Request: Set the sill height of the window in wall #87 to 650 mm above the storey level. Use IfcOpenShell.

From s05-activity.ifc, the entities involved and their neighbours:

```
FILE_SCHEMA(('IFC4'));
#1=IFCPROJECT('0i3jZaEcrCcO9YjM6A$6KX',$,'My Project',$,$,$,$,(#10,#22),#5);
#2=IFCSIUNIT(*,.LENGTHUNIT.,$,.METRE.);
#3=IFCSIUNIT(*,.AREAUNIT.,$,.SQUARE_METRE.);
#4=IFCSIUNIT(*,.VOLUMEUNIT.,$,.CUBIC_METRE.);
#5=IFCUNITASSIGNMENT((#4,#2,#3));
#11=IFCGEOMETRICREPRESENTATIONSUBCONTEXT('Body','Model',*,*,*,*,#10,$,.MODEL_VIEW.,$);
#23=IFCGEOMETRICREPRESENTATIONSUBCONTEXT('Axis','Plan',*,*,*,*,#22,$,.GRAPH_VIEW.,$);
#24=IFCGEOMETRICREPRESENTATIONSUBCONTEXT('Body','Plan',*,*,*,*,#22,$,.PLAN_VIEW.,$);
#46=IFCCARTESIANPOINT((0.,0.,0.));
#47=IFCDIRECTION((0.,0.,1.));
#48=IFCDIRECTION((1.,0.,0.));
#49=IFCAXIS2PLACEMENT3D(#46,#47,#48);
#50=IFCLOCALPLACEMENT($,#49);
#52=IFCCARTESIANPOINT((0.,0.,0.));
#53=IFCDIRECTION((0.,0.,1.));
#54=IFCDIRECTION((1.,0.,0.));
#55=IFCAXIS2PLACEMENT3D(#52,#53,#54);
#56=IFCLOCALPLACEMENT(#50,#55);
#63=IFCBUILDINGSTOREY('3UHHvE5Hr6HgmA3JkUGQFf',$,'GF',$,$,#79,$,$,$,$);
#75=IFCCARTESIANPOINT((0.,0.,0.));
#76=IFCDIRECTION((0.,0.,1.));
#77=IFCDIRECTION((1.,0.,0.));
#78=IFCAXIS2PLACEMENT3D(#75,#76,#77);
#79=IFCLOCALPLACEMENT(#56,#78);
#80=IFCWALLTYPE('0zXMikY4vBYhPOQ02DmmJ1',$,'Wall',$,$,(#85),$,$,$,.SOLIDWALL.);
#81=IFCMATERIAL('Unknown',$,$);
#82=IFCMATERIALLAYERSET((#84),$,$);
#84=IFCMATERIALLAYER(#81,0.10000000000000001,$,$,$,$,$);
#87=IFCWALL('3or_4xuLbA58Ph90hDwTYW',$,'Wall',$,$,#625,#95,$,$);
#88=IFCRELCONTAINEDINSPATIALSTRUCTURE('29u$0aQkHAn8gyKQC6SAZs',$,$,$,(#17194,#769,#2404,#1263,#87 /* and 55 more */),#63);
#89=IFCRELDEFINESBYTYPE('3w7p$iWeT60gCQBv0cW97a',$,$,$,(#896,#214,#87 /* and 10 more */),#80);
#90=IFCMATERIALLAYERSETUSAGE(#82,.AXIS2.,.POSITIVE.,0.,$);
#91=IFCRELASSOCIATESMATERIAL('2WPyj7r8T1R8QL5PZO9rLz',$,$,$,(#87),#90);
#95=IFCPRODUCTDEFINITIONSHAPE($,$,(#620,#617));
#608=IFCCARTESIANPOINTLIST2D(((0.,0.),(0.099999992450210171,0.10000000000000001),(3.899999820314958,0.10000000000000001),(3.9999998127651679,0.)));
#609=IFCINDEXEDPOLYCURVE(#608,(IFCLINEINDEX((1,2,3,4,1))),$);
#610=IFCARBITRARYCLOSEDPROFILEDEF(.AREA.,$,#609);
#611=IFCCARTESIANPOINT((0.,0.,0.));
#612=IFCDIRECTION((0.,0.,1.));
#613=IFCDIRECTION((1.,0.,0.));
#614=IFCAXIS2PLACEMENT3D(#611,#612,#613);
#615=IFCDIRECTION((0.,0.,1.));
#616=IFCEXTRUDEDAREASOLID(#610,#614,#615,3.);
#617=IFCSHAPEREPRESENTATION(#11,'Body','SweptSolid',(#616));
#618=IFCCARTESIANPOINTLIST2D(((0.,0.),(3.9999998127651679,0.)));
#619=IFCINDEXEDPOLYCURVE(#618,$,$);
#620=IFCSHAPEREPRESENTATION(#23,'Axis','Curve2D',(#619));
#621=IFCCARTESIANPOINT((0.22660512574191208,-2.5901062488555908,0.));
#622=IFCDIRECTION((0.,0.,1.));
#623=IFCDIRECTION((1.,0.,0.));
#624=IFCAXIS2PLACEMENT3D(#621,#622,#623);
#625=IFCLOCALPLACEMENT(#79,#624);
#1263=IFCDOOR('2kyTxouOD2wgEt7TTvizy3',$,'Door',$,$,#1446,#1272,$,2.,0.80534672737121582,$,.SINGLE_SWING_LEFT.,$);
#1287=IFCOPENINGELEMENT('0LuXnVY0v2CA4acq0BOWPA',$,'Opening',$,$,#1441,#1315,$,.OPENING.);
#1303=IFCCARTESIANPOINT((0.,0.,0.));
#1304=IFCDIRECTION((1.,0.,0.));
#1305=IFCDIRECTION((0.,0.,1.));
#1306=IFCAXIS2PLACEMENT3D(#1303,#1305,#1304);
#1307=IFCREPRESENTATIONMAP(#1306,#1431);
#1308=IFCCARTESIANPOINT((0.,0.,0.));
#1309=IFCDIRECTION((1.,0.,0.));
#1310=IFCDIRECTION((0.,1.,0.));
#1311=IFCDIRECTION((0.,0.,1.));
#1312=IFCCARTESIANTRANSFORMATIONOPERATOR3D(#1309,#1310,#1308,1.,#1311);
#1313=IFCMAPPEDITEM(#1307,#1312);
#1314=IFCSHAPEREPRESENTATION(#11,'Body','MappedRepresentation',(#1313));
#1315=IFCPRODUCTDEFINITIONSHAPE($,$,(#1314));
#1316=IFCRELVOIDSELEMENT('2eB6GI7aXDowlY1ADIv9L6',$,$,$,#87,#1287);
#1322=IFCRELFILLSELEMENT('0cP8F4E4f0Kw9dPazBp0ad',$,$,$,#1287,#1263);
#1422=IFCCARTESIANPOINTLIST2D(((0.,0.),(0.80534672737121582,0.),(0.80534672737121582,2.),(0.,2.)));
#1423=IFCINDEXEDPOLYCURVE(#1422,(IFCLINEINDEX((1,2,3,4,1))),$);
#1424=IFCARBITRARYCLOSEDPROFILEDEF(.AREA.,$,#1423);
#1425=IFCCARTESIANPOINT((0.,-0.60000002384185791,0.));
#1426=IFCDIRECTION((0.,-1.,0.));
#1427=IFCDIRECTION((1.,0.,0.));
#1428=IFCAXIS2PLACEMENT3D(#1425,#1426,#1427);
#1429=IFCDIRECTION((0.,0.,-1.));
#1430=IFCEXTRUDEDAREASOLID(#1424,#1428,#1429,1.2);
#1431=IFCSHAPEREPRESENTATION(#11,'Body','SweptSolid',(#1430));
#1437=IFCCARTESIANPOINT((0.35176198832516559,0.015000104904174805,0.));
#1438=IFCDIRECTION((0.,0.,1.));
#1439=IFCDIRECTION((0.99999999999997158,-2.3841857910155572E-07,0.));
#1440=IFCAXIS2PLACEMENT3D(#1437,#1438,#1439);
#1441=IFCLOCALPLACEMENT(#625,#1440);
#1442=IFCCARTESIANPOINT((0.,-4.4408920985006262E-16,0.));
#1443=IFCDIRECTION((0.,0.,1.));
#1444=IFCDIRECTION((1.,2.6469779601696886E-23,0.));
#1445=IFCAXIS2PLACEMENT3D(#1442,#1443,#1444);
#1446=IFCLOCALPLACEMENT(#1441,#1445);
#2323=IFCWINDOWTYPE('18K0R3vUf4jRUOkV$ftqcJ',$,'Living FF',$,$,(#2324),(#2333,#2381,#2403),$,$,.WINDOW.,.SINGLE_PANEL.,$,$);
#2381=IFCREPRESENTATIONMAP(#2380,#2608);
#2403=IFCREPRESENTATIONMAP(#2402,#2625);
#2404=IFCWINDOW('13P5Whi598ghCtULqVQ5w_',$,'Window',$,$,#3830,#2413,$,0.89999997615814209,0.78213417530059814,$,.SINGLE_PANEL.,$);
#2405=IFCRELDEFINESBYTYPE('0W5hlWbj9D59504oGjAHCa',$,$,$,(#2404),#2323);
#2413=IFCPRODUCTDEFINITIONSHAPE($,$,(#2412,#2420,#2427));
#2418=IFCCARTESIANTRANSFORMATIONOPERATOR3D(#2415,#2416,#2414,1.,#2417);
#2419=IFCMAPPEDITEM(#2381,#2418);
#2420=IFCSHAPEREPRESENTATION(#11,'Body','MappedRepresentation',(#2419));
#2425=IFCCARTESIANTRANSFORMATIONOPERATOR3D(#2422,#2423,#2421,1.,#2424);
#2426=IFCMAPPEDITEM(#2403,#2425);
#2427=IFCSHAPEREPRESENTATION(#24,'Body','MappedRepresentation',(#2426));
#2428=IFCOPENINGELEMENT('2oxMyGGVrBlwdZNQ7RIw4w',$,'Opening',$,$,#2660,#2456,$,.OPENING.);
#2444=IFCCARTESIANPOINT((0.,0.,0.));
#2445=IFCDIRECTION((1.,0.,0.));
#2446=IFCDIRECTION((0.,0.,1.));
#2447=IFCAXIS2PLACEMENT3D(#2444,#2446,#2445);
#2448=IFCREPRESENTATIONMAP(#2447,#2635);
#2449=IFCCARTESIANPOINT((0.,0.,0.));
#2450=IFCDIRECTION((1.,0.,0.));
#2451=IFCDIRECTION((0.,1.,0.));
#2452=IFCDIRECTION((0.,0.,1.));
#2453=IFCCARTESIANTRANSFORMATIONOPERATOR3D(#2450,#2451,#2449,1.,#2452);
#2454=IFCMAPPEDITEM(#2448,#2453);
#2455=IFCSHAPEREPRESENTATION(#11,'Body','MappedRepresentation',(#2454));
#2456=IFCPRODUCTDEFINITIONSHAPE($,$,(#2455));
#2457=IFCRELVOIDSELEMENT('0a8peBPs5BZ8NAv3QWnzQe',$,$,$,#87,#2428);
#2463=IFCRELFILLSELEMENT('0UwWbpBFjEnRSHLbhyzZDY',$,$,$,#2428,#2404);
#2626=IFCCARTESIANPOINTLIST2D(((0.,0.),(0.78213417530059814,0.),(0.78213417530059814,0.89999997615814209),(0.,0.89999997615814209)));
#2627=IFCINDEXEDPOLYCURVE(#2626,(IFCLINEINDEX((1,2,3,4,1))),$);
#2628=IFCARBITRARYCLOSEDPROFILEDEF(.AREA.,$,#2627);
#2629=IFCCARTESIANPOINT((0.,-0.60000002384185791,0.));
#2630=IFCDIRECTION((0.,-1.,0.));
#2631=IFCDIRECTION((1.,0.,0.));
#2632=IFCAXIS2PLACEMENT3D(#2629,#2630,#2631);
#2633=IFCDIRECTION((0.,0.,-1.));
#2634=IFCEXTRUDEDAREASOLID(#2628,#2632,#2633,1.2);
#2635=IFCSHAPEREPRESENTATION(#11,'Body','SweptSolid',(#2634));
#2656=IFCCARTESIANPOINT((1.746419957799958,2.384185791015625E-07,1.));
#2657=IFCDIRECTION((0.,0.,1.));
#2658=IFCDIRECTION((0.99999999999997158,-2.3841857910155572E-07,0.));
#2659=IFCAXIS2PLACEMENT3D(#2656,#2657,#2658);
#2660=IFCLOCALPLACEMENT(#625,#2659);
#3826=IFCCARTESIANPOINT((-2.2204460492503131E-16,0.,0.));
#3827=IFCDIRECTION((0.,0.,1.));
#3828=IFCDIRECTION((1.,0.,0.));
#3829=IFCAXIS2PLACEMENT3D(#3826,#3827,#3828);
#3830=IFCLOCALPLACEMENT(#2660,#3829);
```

```python
import numpy as np
import ifcopenshell
import ifcopenshell.api.geometry
import ifcopenshell.geom
import ifcopenshell.util.element
import ifcopenshell.util.placement
import ifcopenshell.util.shape
import ifcopenshell.util.unit

model = ifcopenshell.open("s05-activity.ifc")
unit_scale = ifcopenshell.util.unit.calculate_unit_scale(model)

window = model.by_id(2404)
opening = window.FillsVoids[0].RelatingOpeningElement
storey = ifcopenshell.util.element.get_container(window, ifc_class="IfcBuildingStorey")
level = ifcopenshell.util.placement.get_local_placement(storey.ObjectPlacement)[2, 3]

# The opening's origin need not be at the sill, so measure its lowest point.
shape = ifcopenshell.geom.create_shape(ifcopenshell.geom.settings(), opening)
bottom = ifcopenshell.util.shape.get_shape_bottom_elevation(shape, shape.geometry) / unit_scale
dz = level + 0.65 / unit_scale - bottom

shift = np.array([0.0, 0.0, dz])
# The window is placed relative to its opening, so it follows when the opening moves.
matrix = ifcopenshell.util.placement.get_local_placement(opening.ObjectPlacement)
matrix[:3, 3] += shift
ifcopenshell.api.geometry.edit_object_placement(
    model, product=opening, matrix=matrix, is_si=False, should_transform_children=True
)

print(f"moved by {dz * unit_scale:+.3f} m")

model.write("s05-activity_updated.ifc")
```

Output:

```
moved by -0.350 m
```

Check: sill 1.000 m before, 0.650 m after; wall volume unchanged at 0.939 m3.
